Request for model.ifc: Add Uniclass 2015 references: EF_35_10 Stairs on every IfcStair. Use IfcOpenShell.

First a look at what the model holds.

```python
import ifcopenshell

model = ifcopenshell.open("model.ifc")
print(model.schema)
print("classifications:", [c.Name for c in model.by_type("IfcClassification")])
for ifc_class in ("IfcDoor", "IfcRoof", "IfcStair", "IfcWall", "IfcWindow"):
    print(ifc_class, len(model.by_type(ifc_class)))
```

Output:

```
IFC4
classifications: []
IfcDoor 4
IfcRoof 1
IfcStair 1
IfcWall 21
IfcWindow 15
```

```python
import ifcopenshell
import ifcopenshell.api.classification

model = ifcopenshell.open("model.ifc")

system = ifcopenshell.api.classification.add_classification(model, classification="Uniclass 2015")

codes = {
    "IfcStair": ("EF_35_10", "Stairs"),
}
for ifc_class, (code, name) in codes.items():
    products = model.by_type(ifc_class)
    ifcopenshell.api.classification.add_reference(
        model, products=products, classification=system, identification=code, name=name
    )
    print(code, len(products))

model.write("model_updated.ifc")
```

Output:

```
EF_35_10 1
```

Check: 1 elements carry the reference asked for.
